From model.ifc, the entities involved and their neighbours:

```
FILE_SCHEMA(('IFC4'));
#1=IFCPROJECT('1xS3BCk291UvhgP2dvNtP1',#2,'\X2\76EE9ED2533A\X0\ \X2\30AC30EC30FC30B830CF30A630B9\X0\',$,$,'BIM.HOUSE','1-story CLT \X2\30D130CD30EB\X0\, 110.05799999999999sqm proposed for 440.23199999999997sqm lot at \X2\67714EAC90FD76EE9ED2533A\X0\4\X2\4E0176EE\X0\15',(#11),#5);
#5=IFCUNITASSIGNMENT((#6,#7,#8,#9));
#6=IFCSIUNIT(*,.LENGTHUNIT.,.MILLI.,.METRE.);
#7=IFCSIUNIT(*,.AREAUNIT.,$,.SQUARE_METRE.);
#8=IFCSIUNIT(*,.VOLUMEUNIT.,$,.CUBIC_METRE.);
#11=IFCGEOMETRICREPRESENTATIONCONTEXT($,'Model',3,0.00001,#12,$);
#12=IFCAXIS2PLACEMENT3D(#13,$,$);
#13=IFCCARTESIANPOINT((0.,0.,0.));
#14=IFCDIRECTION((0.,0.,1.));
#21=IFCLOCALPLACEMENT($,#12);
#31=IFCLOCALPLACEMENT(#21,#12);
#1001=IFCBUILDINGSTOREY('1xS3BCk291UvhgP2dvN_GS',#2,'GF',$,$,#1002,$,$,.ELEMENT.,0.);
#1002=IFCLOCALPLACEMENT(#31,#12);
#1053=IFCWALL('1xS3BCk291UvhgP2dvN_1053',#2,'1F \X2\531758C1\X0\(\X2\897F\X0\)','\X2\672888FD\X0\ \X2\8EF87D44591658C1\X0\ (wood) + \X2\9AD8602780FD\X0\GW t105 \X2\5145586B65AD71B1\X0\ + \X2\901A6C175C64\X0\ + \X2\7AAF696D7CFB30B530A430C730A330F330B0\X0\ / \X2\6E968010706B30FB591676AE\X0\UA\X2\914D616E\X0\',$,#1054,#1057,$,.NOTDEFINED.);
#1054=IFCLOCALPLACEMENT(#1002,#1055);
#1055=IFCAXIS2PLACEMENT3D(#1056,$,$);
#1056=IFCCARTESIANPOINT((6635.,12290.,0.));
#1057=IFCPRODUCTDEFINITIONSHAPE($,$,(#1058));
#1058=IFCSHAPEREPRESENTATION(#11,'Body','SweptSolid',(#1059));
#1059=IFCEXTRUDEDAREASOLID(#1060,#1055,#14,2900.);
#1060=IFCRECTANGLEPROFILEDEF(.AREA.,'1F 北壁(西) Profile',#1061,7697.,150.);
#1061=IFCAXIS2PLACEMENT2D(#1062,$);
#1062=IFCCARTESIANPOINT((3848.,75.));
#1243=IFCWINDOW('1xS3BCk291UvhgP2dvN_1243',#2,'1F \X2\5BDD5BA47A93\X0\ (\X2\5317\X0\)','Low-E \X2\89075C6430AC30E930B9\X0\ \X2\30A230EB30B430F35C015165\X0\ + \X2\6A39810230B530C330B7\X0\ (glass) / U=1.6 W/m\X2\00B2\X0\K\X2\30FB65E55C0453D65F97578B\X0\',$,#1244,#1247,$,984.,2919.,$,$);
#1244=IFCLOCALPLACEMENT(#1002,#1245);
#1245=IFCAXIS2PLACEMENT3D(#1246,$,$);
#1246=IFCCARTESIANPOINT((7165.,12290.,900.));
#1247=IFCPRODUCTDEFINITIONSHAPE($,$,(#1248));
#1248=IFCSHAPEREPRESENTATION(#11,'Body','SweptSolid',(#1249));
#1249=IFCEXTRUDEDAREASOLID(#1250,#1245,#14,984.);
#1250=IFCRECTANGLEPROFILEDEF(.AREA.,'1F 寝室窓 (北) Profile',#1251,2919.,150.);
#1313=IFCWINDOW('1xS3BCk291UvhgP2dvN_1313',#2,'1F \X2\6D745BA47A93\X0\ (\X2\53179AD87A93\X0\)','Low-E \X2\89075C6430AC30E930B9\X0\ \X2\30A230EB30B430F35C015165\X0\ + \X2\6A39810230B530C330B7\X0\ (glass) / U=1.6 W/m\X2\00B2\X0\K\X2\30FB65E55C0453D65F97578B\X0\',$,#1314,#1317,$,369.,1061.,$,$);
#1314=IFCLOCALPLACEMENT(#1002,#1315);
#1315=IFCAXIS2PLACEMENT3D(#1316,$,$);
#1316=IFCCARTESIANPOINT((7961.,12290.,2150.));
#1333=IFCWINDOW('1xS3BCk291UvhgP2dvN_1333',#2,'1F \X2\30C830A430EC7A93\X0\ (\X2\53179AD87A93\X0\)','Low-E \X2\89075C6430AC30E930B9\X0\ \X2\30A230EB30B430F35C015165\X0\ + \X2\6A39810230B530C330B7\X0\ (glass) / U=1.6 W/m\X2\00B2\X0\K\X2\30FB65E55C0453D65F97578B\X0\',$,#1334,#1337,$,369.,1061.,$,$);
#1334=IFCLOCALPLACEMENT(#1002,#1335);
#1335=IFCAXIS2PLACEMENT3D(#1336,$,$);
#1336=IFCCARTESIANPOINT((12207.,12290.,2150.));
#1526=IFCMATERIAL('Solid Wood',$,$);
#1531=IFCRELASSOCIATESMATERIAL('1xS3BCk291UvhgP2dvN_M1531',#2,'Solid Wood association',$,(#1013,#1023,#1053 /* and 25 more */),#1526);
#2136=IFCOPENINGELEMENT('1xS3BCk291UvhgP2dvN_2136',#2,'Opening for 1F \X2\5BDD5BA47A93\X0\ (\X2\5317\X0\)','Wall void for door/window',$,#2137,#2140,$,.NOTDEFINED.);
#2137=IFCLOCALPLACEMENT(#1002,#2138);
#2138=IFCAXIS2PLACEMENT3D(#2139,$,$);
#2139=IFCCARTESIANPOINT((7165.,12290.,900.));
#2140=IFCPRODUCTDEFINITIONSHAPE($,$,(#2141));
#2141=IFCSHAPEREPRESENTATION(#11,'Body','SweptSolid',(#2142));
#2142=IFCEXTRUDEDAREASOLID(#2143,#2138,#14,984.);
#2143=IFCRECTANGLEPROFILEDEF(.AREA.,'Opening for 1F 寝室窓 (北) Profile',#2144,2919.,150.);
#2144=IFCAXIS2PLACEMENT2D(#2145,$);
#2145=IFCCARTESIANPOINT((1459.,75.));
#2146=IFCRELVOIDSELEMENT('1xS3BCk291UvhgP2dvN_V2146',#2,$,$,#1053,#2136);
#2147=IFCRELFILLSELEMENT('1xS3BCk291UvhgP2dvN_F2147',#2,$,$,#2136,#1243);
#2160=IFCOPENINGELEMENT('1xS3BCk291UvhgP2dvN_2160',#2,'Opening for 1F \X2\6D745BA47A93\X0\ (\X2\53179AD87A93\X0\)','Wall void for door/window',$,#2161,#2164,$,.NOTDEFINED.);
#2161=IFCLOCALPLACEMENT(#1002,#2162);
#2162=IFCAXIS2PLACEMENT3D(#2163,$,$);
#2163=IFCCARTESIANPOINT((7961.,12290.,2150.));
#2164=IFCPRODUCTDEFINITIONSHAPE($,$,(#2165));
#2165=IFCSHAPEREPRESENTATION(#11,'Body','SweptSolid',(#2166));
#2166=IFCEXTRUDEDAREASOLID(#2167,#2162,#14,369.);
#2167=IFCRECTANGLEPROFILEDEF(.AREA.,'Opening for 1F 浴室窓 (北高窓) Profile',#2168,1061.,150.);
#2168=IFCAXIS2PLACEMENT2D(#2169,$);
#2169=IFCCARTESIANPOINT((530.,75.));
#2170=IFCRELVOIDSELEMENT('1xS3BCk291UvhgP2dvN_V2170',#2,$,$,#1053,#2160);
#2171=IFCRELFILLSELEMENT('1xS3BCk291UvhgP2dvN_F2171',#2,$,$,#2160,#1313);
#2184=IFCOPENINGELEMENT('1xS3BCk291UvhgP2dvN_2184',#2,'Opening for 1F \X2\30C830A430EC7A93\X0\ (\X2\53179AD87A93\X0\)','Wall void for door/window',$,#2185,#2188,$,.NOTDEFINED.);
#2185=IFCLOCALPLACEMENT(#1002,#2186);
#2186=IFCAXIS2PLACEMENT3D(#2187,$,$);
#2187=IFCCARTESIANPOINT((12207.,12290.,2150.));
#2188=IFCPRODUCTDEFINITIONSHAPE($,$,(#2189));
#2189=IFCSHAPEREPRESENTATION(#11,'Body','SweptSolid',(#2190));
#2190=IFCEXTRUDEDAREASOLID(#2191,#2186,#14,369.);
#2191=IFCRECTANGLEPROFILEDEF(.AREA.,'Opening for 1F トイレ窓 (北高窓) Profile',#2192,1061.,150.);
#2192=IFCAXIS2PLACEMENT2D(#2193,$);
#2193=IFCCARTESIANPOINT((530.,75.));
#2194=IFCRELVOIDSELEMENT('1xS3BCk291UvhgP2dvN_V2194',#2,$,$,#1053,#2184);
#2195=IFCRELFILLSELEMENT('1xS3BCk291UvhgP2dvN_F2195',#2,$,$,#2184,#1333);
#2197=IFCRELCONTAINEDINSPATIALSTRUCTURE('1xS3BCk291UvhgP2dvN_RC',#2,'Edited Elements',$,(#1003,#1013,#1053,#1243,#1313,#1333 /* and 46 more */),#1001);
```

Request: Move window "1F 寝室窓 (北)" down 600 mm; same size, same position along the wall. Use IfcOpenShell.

```python
import numpy as np
import ifcopenshell
import ifcopenshell.api.geometry
import ifcopenshell.util.placement
import ifcopenshell.util.unit

model = ifcopenshell.open("model.ifc")
unit_scale = ifcopenshell.util.unit.calculate_unit_scale(model)

window = model.by_id(1243)
opening = window.FillsVoids[0].RelatingOpeningElement
dz = -0.6 / unit_scale

shift = np.array([0.0, 0.0, dz])
# The window is not placed relative to its opening, so move both.
for product in (opening, window):
    matrix = ifcopenshell.util.placement.get_local_placement(product.ObjectPlacement)
    matrix[:3, 3] += shift
    ifcopenshell.api.geometry.edit_object_placement(model, product=product, matrix=matrix, is_si=False)

print(f"moved by {dz * unit_scale:+.3f} m")

model.write("model-out.ifc")
```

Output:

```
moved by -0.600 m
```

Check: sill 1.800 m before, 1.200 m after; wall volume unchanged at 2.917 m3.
